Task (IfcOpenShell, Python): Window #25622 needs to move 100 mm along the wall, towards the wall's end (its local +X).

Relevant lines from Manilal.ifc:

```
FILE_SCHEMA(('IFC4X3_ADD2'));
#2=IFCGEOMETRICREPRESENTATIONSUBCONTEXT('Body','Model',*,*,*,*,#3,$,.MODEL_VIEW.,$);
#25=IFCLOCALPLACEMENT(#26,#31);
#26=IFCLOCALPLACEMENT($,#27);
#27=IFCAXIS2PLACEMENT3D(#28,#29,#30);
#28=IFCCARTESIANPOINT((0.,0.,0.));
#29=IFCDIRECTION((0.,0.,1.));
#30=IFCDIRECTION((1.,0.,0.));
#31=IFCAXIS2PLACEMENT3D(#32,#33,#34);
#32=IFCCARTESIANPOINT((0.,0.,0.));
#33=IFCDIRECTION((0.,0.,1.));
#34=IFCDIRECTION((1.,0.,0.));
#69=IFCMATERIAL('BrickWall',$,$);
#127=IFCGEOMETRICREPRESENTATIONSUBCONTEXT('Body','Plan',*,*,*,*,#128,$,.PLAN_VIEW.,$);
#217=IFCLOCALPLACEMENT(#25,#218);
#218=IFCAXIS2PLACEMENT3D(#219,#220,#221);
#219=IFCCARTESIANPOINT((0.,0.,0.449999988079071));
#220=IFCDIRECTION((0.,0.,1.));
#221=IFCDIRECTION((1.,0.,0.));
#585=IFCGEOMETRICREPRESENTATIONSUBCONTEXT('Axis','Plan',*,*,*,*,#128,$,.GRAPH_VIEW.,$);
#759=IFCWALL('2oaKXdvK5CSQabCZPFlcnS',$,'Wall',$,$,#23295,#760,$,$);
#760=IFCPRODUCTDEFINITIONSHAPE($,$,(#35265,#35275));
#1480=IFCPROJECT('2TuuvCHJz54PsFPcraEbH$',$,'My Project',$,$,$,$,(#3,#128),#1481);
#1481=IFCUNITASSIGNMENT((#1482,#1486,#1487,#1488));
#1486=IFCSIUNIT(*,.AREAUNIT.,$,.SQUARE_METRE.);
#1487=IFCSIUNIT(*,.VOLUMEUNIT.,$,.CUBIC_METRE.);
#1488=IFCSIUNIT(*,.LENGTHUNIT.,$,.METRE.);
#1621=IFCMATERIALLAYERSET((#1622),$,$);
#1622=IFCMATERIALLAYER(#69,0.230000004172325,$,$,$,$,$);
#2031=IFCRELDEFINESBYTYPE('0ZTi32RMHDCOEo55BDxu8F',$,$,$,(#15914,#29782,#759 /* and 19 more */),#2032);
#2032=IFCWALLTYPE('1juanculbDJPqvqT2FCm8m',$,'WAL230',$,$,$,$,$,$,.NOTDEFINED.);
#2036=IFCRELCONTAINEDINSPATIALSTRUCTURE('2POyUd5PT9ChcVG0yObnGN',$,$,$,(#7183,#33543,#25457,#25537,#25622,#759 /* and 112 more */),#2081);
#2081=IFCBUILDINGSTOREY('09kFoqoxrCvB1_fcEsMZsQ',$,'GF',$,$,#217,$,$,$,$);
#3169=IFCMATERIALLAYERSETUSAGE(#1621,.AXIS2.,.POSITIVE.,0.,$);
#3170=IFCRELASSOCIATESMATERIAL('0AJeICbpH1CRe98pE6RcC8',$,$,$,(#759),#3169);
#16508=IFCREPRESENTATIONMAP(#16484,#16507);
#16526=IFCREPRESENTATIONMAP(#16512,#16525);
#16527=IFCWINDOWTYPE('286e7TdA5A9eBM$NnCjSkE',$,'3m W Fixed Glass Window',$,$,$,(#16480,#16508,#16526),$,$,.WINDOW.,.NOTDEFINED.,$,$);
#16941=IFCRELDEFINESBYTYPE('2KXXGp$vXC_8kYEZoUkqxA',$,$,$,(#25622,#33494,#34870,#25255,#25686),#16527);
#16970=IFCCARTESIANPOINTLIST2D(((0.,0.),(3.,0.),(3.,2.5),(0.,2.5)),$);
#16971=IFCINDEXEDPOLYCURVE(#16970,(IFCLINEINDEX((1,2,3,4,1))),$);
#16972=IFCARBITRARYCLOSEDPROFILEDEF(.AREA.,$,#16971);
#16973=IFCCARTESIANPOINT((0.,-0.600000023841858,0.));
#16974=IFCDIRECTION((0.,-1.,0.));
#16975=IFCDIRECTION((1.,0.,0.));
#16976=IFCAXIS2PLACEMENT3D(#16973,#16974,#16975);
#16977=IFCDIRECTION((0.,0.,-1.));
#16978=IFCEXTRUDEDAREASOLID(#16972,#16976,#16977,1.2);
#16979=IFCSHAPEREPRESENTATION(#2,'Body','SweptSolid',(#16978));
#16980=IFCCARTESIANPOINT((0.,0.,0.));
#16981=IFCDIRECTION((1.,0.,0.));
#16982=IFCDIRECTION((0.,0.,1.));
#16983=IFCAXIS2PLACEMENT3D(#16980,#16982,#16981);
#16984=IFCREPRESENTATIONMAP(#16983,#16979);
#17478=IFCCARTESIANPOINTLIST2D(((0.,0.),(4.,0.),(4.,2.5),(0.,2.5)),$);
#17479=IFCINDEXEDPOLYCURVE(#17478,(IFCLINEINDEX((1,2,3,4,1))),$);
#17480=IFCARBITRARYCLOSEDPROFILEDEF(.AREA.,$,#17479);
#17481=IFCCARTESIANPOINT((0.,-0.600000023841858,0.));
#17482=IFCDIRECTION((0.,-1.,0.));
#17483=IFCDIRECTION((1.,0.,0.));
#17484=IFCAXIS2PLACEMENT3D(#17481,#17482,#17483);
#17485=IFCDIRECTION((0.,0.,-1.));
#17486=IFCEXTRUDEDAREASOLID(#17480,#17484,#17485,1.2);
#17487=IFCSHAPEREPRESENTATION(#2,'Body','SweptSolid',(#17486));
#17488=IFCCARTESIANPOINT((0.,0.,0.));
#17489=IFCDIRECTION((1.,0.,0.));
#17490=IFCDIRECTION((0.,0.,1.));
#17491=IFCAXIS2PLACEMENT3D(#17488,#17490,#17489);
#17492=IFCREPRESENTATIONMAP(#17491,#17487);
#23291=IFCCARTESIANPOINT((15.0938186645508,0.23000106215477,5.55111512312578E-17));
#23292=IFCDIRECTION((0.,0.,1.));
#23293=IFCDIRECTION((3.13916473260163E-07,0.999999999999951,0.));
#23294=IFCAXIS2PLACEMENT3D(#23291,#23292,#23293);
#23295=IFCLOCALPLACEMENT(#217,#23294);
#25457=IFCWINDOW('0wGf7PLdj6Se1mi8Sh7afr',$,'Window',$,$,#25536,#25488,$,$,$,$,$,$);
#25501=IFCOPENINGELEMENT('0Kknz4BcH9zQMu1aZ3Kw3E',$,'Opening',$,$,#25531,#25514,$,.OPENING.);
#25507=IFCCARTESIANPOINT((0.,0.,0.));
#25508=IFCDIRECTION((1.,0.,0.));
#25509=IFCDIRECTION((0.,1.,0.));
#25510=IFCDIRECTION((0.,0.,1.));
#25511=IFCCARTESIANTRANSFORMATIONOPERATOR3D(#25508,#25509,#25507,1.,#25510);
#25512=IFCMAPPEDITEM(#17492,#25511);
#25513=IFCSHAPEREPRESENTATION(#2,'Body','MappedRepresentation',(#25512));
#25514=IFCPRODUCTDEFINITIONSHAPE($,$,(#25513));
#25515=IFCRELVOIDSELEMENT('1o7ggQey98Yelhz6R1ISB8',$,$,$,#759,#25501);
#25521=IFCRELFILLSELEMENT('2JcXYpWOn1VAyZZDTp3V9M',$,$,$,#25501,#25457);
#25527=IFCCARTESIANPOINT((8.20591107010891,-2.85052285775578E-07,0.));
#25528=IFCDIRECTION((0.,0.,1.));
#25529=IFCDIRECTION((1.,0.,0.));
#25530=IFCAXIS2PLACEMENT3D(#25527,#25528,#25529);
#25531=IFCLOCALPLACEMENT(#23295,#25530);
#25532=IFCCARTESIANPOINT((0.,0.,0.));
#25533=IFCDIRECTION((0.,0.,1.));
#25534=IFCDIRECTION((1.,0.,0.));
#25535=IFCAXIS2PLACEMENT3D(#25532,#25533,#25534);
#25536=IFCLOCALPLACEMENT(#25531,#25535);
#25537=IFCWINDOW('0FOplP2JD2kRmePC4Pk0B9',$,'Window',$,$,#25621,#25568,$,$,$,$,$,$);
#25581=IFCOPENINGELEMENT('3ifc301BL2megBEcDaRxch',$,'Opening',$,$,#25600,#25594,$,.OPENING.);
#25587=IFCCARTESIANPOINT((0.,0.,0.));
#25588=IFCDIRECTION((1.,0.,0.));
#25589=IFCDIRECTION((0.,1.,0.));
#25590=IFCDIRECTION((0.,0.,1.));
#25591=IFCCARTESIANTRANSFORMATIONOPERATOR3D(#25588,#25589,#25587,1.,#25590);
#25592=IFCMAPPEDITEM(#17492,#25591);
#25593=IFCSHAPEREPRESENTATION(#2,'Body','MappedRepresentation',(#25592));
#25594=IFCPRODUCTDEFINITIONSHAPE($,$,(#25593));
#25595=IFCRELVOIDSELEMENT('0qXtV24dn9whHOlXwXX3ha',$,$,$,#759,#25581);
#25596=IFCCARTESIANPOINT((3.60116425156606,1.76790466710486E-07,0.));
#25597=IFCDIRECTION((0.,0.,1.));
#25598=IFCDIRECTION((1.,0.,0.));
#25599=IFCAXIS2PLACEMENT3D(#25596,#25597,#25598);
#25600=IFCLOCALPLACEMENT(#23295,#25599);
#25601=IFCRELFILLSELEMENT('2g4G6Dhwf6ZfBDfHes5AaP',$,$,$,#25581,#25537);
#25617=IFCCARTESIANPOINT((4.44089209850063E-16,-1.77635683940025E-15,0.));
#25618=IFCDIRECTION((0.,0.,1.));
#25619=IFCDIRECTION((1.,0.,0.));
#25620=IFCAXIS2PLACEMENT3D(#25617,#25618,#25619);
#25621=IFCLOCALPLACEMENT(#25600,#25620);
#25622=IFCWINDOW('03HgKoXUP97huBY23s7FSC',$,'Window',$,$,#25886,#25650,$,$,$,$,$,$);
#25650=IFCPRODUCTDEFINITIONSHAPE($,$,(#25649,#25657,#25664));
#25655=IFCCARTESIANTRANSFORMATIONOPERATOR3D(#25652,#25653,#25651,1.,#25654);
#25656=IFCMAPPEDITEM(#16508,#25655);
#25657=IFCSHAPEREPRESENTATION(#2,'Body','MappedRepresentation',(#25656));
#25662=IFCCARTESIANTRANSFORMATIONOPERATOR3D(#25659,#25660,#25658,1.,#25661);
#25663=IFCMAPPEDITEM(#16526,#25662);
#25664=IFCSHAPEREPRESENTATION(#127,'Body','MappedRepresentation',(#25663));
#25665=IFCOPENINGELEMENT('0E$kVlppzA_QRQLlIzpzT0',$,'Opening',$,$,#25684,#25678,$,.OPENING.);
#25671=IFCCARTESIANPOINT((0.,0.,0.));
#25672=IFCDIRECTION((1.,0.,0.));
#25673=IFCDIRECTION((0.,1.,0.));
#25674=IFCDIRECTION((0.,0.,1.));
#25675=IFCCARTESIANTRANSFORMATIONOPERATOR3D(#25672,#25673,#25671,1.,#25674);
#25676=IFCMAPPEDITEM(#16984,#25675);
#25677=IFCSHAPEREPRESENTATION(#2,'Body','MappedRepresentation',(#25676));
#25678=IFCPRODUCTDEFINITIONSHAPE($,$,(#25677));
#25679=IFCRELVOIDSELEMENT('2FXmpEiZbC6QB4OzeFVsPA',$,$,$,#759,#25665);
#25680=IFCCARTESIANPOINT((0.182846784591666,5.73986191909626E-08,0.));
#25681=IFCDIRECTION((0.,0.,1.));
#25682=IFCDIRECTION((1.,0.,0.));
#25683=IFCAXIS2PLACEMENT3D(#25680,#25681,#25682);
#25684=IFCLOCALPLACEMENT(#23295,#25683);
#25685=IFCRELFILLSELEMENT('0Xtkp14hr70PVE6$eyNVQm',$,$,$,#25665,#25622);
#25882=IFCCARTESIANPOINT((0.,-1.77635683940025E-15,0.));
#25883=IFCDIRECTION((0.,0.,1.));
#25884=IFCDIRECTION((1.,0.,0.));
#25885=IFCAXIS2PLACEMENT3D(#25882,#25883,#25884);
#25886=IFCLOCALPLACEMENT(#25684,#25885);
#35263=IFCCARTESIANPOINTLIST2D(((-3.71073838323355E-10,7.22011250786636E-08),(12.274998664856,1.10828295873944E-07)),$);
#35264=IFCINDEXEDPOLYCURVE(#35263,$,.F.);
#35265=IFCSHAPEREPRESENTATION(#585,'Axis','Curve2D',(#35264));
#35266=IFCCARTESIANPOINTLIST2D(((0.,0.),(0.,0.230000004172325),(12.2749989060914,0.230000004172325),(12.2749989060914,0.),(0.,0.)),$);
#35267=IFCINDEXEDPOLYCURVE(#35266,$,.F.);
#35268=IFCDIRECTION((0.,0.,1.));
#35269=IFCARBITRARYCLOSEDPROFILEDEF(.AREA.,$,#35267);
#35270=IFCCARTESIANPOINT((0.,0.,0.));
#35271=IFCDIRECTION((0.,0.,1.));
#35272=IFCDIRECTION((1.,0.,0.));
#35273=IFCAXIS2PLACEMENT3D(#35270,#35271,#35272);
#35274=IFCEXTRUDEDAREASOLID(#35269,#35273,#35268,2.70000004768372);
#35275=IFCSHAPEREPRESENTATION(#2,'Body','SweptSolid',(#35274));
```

```python
import ifcopenshell
import ifcopenshell.api.geometry
import ifcopenshell.util.placement
import ifcopenshell.util.unit

model = ifcopenshell.open("Manilal.ifc")
unit_scale = ifcopenshell.util.unit.calculate_unit_scale(model)

window = model.by_id(25622)
opening = window.FillsVoids[0].RelatingOpeningElement
wall = opening.VoidsElements[0].RelatingBuildingElement

wall_matrix = ifcopenshell.util.placement.get_local_placement(wall.ObjectPlacement)
shift = wall_matrix[:3, 0] * 0.1 / unit_scale
before = ifcopenshell.util.placement.get_local_placement(window.ObjectPlacement)[:3, 3].copy()

# The window is placed relative to its opening, so it follows when the opening moves.
matrix = ifcopenshell.util.placement.get_local_placement(opening.ObjectPlacement)
matrix[:3, 3] += shift
ifcopenshell.api.geometry.edit_object_placement(
    model, product=opening, matrix=matrix, is_si=False, should_transform_children=True
)

after = ifcopenshell.util.placement.get_local_placement(window.ObjectPlacement)[:3, 3]
print("window moved by", (after - before).round(3) + 0.0)

model.write("Manilal-out.ifc")
```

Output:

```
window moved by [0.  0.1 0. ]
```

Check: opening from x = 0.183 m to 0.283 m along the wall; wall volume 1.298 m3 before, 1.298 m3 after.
